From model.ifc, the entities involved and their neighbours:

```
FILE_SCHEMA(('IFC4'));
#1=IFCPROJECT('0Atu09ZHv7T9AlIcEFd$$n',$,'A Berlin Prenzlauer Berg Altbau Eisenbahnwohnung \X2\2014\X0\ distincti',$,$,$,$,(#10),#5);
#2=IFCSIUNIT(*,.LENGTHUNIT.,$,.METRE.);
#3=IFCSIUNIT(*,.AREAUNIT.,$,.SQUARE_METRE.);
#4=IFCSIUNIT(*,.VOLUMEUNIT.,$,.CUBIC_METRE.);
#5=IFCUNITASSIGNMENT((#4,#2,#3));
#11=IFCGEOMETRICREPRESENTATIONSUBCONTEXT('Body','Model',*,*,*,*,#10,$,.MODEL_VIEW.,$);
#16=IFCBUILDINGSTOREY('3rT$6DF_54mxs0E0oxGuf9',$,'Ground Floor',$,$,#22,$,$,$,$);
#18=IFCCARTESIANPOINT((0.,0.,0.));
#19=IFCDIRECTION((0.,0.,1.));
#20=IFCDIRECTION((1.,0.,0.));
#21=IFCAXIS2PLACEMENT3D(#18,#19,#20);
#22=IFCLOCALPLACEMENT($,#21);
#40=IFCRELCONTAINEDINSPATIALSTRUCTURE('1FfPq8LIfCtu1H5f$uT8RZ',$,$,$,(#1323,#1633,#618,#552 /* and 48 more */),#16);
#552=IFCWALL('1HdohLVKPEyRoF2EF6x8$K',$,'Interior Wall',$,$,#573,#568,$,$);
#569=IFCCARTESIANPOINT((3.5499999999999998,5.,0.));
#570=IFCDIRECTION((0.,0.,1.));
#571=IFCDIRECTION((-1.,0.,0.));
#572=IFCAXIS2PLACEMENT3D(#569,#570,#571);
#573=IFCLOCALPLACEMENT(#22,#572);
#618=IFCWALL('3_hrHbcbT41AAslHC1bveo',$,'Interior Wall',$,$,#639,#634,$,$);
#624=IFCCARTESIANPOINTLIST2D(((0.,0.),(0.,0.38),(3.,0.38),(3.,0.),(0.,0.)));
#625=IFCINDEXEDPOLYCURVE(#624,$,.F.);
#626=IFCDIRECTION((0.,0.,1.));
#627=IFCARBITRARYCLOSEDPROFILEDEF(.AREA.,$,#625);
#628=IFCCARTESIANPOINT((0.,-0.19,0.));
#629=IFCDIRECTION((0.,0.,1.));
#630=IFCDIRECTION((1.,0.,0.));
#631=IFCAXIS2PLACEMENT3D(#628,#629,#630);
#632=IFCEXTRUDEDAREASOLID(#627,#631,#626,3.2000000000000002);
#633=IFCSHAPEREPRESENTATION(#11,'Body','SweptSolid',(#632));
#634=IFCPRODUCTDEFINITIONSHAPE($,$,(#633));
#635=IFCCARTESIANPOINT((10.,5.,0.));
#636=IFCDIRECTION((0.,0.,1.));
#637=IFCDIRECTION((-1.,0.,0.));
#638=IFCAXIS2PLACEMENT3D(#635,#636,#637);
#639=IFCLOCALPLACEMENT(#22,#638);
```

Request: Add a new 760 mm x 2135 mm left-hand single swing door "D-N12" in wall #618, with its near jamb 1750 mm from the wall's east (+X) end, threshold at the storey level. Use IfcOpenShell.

```python
import numpy as np
import ifcopenshell
import ifcopenshell.api.feature
import ifcopenshell.api.geometry
import ifcopenshell.api.root
import ifcopenshell.api.spatial
import ifcopenshell.geom
import ifcopenshell.util.element
import ifcopenshell.util.placement
import ifcopenshell.util.representation
import ifcopenshell.util.shape
import ifcopenshell.util.unit

model = ifcopenshell.open("model.ifc")
unit_scale = ifcopenshell.util.unit.calculate_unit_scale(model)
settings = ifcopenshell.geom.settings()


def volume(element):
    """Net volume in cubic metres, openings subtracted."""
    shape = ifcopenshell.geom.create_shape(settings, element)
    return ifcopenshell.util.shape.get_volume(shape.geometry)


wall = model.by_guid("3_hrHbcbT41AAslHC1bveo")
storey = ifcopenshell.util.element.get_container(wall, ifc_class="IfcBuildingStorey")
context = ifcopenshell.util.representation.get_context(model, "Model", "Body", "MODEL_VIEW")
before = volume(wall)

width, height, from_end, sill = 0.76, 2.135, 1.75, 0.0  # metres

# The wall runs along its own X axis, and the end named is its -X end.
wall_shape = ifcopenshell.geom.create_shape(settings, wall)
x, y, z = ifcopenshell.util.shape.get_vertices(wall_shape.geometry).T
start = x.min() + from_end
face, thickness = float(y.min()), float(y.max() - y.min())
wall_matrix = ifcopenshell.util.placement.get_local_placement(wall.ObjectPlacement)
level = ifcopenshell.util.placement.get_local_placement(storey.ObjectPlacement)[2, 3]


def in_wall(x, y):
    """Placement at x, y metres in the wall's axes, at sill height."""
    matrix = wall_matrix.copy()
    matrix[:, 3] = wall_matrix @ np.array([x / unit_scale, y / unit_scale, 0.0, 1.0])
    matrix[2, 3] = level + sill / unit_scale
    return matrix


# Opening: a box that overshoots both wall faces by 50 mm.
opening = ifcopenshell.api.root.create_entity(model, ifc_class="IfcOpeningElement", predefined_type="OPENING")
box = ifcopenshell.api.geometry.add_wall_representation(
    model, context=context, length=width, height=height, thickness=thickness + 0.1
)
ifcopenshell.api.geometry.assign_representation(model, product=opening, representation=box)
ifcopenshell.api.geometry.edit_object_placement(model, product=opening, matrix=in_wall(start, face - 0.05), is_si=False)
ifcopenshell.api.feature.add_feature(model, feature=opening, element=wall)

door = ifcopenshell.api.root.create_entity(model, ifc_class="IfcDoor", name="D-N12", predefined_type="DOOR")
door.OverallWidth, door.OverallHeight = width / unit_scale, height / unit_scale
door.OperationType = "SINGLE_SWING_LEFT"
body = ifcopenshell.api.geometry.add_door_representation(
    model,
    context=context,
    overall_width=door.OverallWidth,
    overall_height=door.OverallHeight,
    operation_type="SINGLE_SWING_LEFT",
    lining_properties={"LiningDepth": thickness / unit_scale, "ThresholdDepth": thickness / unit_scale},
)
ifcopenshell.api.geometry.assign_representation(model, product=door, representation=body)
ifcopenshell.api.spatial.assign_container(model, products=[door], relating_structure=storey)
ifcopenshell.api.feature.add_filling(model, opening=opening, element=door)

# The lining spans the wall, so the door starts at the wall face.
ifcopenshell.api.geometry.edit_object_placement(model, product=door, matrix=in_wall(start, face), is_si=False)

after = volume(wall)

print(f"wall volume {before:.3f} -> {after:.3f} m3")

model.write("model-out.ifc")
```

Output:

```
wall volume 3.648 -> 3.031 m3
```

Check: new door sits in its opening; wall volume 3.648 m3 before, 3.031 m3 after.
